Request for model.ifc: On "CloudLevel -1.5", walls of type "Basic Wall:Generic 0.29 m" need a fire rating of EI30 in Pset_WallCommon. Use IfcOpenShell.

First a look at what the model holds.

```python
import ifcopenshell
import ifcopenshell.util.element

model = ifcopenshell.open("model.ifc")
print(model.schema)
storey = next(s for s in model.by_type("IfcBuildingStorey") if s.Name == "CloudLevel -1.5")
walls = [e for e in ifcopenshell.util.element.get_decomposition(storey) if e.is_a("IfcWall")]
seen = {}
for e in walls:
    element_type = ifcopenshell.util.element.get_type(e)
    key = (element_type.Name if element_type != e and element_type else None, ifcopenshell.util.element.get_pset(e, "Pset_WallCommon", "FireRating"))
    seen[key] = seen.get(key, 0) + 1
for (name, value), count in sorted(seen.items(), key=str):
    print(count, "x", name, "|", value)
```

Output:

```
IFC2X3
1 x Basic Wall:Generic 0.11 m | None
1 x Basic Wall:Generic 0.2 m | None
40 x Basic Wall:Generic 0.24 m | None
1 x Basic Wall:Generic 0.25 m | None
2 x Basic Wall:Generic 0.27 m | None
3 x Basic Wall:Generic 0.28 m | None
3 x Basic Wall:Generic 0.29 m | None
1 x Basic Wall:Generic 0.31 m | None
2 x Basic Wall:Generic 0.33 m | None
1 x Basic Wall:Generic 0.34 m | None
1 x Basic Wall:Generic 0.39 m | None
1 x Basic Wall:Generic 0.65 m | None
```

```python
import ifcopenshell
import ifcopenshell.api.pset
import ifcopenshell.util.element

model = ifcopenshell.open("model.ifc")

storey = next(s for s in model.by_type("IfcBuildingStorey") if s.Name == "CloudLevel -1.5")
walls = [e for e in ifcopenshell.util.element.get_decomposition(storey) if e.is_a("IfcWall")]

count = 0
for e in walls:
    element_type = ifcopenshell.util.element.get_type(e)
    if element_type in (None, e) or element_type.Name != "Basic Wall:Generic 0.29 m":
        continue
    # add_pset returns the element's existing set when there is one.
    pset = ifcopenshell.api.pset.add_pset(model, product=e, name="Pset_WallCommon")
    ifcopenshell.api.pset.edit_pset(model, pset=pset, properties={"FireRating": "EI30"})
    count += 1

print(count, "walls updated")

model.write("model_edited.ifc")
```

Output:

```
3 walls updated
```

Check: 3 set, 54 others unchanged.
